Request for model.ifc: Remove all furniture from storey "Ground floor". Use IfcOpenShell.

First a look at what the model holds.

```python
import ifcopenshell
import ifcopenshell.util.element

model = ifcopenshell.open("model.ifc")
print(model.schema)
storey = next(s for s in model.by_type("IfcBuildingStorey") if s.Name == "Ground floor")
furniture = [e for e in ifcopenshell.util.element.get_decomposition(storey) if e.is_a("IfcFurnishingElement")]
seen = {}
for e in furniture:
    element_type = ifcopenshell.util.element.get_type(e)
    name = element_type.Name if element_type not in (None, e) else None
    seen[name] = seen.get(name, 0) + 1
for name, count in sorted(seen.items(), key=str):
    print(count, "x", name)
```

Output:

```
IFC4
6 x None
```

```python
import ifcopenshell
import ifcopenshell.api.root
import ifcopenshell.util.element

model = ifcopenshell.open("model.ifc")

storey = next(s for s in model.by_type("IfcBuildingStorey") if s.Name == "Ground floor")
furniture = [e for e in ifcopenshell.util.element.get_decomposition(storey) if e.is_a("IfcFurnishingElement")]

for e in furniture:
    ifcopenshell.api.root.remove_product(model, product=e)
print(len(furniture), "removed")

model.write("model_updated.ifc")
```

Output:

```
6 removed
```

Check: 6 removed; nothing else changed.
